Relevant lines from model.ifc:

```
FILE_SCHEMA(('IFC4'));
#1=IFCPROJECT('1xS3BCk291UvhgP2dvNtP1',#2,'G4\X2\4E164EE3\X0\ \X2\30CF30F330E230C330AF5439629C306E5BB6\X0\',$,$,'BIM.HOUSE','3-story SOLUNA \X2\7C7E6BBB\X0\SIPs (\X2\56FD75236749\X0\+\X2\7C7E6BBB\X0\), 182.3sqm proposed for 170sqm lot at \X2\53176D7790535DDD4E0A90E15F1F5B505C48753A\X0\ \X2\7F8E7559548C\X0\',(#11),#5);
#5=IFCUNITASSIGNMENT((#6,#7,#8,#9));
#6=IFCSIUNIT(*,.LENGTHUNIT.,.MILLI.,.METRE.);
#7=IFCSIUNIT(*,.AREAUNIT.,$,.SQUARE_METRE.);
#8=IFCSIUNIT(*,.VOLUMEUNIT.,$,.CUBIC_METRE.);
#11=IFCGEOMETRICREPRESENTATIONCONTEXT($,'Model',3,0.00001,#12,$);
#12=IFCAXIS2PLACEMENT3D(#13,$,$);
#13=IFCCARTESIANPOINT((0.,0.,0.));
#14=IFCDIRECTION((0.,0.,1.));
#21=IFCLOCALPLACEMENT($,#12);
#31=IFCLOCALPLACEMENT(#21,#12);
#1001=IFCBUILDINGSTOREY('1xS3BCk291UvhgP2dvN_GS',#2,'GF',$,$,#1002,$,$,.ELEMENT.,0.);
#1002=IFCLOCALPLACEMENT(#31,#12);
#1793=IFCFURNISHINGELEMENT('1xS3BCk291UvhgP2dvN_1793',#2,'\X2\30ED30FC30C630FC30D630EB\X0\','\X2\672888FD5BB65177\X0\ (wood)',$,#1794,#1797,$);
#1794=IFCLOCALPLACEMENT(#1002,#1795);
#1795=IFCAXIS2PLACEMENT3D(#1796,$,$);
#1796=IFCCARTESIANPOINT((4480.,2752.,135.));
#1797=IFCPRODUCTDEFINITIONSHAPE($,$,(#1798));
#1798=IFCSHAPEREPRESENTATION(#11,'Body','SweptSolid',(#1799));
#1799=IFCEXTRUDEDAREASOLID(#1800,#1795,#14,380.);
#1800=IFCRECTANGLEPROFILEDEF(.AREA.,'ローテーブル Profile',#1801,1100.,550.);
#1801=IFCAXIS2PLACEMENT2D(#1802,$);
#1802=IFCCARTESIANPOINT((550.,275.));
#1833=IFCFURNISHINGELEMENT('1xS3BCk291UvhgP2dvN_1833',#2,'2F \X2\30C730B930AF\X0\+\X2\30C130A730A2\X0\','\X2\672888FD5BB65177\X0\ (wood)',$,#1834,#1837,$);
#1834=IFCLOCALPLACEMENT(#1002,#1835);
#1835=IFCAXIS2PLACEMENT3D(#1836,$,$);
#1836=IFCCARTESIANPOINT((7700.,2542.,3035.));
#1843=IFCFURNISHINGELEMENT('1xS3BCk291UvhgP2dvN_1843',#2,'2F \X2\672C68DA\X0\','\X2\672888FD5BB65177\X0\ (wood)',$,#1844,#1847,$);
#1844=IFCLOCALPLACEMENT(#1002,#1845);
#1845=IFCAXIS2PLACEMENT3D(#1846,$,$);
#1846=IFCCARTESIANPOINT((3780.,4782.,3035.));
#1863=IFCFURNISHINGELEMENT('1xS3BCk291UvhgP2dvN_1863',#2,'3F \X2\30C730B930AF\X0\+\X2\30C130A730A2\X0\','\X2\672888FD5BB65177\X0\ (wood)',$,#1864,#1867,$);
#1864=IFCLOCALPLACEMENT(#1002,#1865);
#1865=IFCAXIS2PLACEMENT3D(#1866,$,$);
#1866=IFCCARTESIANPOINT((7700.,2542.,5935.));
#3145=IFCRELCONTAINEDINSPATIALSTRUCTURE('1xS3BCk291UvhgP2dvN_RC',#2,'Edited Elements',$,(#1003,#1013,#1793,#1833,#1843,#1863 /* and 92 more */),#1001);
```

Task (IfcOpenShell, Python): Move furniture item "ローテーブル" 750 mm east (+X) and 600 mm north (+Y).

```python
import ifcopenshell
import ifcopenshell.api.geometry
import ifcopenshell.util.placement

model = ifcopenshell.open("model.ifc")

item = model.by_guid("1xS3BCk291UvhgP2dvN_1793")
matrix = ifcopenshell.util.placement.get_local_placement(item.ObjectPlacement)
matrix[0, 3] += 750.0
matrix[1, 3] += 600.0
ifcopenshell.api.geometry.edit_object_placement(model, product=item, matrix=matrix, is_si=False)

print(ifcopenshell.util.placement.get_local_placement(item.ObjectPlacement).round(3) + 0.0)

model.write("model-out.ifc")
```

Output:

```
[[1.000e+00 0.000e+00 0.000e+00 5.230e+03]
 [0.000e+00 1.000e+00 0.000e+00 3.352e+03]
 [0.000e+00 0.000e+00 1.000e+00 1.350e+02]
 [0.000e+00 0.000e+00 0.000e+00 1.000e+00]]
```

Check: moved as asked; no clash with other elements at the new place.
